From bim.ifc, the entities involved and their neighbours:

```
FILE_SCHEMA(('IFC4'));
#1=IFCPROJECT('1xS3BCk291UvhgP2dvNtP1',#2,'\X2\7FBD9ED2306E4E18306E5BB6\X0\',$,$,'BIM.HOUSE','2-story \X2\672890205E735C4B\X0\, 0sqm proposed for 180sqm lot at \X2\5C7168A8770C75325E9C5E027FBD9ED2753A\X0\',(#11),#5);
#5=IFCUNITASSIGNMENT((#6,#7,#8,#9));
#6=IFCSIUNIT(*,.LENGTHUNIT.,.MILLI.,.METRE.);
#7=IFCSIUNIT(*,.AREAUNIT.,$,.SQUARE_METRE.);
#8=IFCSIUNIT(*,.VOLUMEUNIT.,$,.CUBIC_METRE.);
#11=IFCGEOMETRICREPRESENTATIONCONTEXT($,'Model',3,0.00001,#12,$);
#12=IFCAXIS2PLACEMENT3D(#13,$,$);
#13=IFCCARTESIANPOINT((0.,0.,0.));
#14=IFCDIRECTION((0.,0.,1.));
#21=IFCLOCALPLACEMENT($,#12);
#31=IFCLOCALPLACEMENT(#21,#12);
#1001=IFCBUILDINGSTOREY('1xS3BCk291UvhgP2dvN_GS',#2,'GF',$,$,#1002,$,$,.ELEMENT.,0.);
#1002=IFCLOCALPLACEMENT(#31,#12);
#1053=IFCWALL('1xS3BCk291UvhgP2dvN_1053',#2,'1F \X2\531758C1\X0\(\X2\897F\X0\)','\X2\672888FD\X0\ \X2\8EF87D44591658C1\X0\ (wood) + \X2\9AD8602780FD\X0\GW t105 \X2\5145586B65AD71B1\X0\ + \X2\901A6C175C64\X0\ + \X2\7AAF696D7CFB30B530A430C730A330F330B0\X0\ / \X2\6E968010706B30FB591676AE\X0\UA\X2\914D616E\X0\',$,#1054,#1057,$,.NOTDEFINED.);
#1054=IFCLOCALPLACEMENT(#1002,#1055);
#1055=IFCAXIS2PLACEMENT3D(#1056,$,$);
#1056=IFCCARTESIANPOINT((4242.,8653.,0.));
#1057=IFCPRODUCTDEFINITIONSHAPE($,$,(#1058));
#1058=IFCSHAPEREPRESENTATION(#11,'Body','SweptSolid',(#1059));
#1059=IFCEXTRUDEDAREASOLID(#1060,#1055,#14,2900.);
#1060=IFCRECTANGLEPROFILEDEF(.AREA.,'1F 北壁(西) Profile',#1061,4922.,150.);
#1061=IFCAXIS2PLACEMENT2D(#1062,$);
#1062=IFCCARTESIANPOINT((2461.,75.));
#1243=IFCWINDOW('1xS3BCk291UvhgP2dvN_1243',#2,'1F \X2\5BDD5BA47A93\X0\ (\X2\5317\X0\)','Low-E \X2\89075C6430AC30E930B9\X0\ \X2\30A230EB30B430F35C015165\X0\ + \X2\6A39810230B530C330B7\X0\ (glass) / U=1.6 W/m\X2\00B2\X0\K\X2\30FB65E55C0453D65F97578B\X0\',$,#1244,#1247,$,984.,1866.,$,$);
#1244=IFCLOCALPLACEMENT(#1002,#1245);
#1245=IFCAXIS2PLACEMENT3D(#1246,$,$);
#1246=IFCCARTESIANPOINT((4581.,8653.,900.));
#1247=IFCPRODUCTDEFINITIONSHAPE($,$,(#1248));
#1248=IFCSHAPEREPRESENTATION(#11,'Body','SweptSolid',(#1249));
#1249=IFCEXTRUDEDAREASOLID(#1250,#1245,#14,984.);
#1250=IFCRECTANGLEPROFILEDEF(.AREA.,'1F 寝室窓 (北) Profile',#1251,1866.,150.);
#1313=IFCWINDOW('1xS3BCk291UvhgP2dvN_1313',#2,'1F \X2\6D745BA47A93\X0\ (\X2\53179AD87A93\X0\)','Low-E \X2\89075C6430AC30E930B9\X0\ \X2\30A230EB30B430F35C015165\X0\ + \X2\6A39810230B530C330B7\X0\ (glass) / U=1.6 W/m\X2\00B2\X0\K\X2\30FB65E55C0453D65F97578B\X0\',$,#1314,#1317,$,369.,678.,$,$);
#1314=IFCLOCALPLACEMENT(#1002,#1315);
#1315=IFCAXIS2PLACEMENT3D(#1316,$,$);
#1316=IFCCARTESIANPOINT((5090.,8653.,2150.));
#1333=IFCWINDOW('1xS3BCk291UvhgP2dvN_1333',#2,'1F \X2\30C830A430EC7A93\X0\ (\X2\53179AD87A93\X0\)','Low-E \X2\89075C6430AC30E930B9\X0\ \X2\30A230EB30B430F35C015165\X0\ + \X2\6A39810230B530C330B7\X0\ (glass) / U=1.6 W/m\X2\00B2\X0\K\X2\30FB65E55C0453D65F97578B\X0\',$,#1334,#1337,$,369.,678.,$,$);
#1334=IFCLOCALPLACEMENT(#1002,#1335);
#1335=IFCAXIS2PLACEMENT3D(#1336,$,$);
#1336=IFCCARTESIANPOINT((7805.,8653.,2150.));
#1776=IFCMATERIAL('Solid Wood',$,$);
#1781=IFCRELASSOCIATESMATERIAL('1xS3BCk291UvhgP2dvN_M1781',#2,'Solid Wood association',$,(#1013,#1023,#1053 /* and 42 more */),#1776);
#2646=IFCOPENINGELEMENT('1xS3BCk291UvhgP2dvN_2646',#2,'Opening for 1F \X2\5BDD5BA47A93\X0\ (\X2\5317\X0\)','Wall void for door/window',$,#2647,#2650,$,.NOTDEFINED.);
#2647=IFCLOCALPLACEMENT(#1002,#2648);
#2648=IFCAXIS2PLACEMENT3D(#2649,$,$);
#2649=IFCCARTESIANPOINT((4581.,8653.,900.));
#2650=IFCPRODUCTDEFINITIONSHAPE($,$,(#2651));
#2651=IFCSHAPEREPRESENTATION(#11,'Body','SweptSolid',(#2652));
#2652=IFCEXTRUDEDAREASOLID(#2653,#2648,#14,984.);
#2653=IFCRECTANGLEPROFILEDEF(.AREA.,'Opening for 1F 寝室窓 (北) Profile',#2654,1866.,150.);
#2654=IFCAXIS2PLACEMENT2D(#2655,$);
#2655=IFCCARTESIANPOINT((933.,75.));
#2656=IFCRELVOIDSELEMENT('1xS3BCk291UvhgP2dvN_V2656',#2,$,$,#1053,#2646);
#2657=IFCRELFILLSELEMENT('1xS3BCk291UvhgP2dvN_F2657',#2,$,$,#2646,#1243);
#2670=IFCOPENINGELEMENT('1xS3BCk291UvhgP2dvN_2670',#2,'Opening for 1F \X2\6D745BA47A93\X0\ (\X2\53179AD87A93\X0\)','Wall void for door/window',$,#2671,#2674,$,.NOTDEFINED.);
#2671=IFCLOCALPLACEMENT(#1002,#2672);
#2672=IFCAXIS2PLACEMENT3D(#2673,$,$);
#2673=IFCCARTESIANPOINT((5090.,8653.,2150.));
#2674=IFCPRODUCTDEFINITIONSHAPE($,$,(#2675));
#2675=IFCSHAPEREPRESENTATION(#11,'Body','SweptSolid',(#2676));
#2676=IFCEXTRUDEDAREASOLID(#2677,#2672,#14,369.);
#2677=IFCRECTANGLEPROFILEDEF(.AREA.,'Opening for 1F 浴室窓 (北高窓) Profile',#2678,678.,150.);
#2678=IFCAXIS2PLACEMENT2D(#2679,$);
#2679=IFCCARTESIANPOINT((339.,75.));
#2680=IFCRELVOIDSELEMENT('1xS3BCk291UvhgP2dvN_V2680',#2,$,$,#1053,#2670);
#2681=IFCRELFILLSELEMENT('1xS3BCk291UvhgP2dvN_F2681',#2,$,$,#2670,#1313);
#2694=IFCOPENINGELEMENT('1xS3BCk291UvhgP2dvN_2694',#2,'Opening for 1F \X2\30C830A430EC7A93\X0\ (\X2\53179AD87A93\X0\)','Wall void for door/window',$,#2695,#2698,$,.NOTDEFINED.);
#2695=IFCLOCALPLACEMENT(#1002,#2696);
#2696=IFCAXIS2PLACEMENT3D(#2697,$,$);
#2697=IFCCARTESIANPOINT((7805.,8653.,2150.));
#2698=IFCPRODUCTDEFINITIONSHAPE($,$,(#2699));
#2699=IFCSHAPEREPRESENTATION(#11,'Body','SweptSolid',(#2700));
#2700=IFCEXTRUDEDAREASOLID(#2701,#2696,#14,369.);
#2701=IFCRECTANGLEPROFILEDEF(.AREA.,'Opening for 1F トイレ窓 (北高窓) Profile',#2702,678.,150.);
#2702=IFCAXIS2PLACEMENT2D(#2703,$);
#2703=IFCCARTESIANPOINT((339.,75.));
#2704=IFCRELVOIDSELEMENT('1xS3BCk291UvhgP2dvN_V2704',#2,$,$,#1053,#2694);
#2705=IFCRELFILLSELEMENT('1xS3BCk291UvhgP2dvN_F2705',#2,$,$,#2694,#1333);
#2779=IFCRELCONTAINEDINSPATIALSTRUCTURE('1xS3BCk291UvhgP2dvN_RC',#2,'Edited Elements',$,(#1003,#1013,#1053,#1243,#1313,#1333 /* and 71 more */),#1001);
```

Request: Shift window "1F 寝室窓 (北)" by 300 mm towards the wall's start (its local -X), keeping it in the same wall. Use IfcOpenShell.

```python
import ifcopenshell
import ifcopenshell.api.geometry
import ifcopenshell.util.placement
import ifcopenshell.util.unit

model = ifcopenshell.open("bim.ifc")
unit_scale = ifcopenshell.util.unit.calculate_unit_scale(model)

window = model.by_guid("1xS3BCk291UvhgP2dvN_1243")
opening = window.FillsVoids[0].RelatingOpeningElement
wall = opening.VoidsElements[0].RelatingBuildingElement

wall_matrix = ifcopenshell.util.placement.get_local_placement(wall.ObjectPlacement)
shift = wall_matrix[:3, 0] * -0.3 / unit_scale
before = ifcopenshell.util.placement.get_local_placement(window.ObjectPlacement)[:3, 3].copy()

# The window is not placed relative to its opening, so move both.
for product in (opening, window):
    matrix = ifcopenshell.util.placement.get_local_placement(product.ObjectPlacement)
    matrix[:3, 3] += shift
    ifcopenshell.api.geometry.edit_object_placement(model, product=product, matrix=matrix, is_si=False)

after = ifcopenshell.util.placement.get_local_placement(window.ObjectPlacement)[:3, 3]
print("window moved by", (after - before).round(3) + 0.0)

model.write("bim_edited.ifc")
```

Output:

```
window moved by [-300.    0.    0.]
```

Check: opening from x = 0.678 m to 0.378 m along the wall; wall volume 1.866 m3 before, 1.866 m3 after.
